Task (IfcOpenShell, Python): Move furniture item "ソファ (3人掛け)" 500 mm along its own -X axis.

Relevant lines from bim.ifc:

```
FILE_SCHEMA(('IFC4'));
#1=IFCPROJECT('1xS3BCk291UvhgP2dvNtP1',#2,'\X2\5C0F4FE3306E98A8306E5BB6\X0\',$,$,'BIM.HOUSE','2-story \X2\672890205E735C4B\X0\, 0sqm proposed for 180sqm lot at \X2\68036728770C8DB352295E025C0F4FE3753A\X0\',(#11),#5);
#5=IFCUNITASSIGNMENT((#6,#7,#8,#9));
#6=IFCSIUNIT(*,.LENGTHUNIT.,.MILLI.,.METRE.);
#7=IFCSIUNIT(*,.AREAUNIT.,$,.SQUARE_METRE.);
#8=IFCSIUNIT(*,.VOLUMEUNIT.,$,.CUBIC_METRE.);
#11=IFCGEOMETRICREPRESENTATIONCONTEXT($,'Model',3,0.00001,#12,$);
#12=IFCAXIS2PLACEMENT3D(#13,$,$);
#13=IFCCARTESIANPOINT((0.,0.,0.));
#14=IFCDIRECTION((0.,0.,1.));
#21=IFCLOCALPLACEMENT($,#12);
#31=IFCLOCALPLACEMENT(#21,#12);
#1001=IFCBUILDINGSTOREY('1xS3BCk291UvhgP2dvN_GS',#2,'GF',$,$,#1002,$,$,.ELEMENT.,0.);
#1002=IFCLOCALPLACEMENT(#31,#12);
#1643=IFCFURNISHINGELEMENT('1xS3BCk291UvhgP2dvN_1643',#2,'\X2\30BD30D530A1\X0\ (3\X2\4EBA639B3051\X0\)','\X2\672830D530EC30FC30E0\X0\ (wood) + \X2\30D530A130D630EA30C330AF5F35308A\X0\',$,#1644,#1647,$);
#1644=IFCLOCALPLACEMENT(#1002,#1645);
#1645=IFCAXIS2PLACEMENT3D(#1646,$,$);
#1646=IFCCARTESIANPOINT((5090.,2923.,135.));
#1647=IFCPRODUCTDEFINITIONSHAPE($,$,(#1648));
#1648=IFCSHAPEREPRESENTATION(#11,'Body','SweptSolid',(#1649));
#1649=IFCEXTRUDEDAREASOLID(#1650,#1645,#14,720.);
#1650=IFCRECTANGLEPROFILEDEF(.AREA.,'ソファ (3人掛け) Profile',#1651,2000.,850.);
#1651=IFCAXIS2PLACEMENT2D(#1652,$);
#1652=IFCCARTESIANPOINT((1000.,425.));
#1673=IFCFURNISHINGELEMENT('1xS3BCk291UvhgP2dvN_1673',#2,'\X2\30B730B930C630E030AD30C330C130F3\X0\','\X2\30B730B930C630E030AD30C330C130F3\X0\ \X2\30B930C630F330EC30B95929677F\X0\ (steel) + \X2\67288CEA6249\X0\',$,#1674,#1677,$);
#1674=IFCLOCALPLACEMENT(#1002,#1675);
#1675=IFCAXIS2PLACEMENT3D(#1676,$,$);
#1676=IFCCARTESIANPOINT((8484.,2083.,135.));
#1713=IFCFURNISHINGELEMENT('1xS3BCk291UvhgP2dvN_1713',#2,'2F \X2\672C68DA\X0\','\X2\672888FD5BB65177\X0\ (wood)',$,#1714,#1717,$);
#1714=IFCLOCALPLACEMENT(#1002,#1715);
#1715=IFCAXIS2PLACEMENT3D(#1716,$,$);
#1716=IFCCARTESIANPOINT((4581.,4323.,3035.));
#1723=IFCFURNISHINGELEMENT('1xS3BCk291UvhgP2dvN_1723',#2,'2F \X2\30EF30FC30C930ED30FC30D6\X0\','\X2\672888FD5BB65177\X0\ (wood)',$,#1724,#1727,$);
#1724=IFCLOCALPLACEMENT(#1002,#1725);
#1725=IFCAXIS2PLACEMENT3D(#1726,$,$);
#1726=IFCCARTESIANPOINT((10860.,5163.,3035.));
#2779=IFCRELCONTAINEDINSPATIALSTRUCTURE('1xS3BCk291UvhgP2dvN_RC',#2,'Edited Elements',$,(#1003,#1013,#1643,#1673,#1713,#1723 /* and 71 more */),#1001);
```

```python
import ifcopenshell
import ifcopenshell.api.geometry
import ifcopenshell.util.placement
import ifcopenshell.util.unit

model = ifcopenshell.open("bim.ifc")
unit_scale = ifcopenshell.util.unit.calculate_unit_scale(model)

item = model.by_guid("1xS3BCk291UvhgP2dvN_1643")
matrix = ifcopenshell.util.placement.get_local_placement(item.ObjectPlacement)
matrix[:3, 3] -= matrix[:3, 0] * 0.5 / unit_scale
ifcopenshell.api.geometry.edit_object_placement(model, product=item, matrix=matrix, is_si=False)

print(ifcopenshell.util.placement.get_local_placement(item.ObjectPlacement).round(3) + 0.0)

model.write("bim-out.ifc")
```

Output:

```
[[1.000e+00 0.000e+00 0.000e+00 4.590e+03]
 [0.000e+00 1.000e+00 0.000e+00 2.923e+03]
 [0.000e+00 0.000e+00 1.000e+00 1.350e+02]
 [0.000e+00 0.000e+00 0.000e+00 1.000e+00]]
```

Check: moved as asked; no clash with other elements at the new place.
